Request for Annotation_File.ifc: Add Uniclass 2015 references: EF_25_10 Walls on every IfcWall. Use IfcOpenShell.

First a look at what the model holds.

```python
import ifcopenshell

model = ifcopenshell.open("Annotation_File.ifc")
print(model.schema)
print("classifications:", [c.Name for c in model.by_type("IfcClassification")])
for ifc_class in ("IfcDoor", "IfcRoof", "IfcStair", "IfcWall", "IfcWindow"):
    print(ifc_class, len(model.by_type(ifc_class)))
```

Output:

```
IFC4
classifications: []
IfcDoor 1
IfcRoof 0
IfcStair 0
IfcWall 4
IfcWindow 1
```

```python
import ifcopenshell
import ifcopenshell.api.classification

model = ifcopenshell.open("Annotation_File.ifc")

system = ifcopenshell.api.classification.add_classification(model, classification="Uniclass 2015")

codes = {
    "IfcWall": ("EF_25_10", "Walls"),
}
for ifc_class, (code, name) in codes.items():
    products = model.by_type(ifc_class)
    ifcopenshell.api.classification.add_reference(
        model, products=products, classification=system, identification=code, name=name
    )
    print(code, len(products))

model.write("Annotation_File_edited.ifc")
```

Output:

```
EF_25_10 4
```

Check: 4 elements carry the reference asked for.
